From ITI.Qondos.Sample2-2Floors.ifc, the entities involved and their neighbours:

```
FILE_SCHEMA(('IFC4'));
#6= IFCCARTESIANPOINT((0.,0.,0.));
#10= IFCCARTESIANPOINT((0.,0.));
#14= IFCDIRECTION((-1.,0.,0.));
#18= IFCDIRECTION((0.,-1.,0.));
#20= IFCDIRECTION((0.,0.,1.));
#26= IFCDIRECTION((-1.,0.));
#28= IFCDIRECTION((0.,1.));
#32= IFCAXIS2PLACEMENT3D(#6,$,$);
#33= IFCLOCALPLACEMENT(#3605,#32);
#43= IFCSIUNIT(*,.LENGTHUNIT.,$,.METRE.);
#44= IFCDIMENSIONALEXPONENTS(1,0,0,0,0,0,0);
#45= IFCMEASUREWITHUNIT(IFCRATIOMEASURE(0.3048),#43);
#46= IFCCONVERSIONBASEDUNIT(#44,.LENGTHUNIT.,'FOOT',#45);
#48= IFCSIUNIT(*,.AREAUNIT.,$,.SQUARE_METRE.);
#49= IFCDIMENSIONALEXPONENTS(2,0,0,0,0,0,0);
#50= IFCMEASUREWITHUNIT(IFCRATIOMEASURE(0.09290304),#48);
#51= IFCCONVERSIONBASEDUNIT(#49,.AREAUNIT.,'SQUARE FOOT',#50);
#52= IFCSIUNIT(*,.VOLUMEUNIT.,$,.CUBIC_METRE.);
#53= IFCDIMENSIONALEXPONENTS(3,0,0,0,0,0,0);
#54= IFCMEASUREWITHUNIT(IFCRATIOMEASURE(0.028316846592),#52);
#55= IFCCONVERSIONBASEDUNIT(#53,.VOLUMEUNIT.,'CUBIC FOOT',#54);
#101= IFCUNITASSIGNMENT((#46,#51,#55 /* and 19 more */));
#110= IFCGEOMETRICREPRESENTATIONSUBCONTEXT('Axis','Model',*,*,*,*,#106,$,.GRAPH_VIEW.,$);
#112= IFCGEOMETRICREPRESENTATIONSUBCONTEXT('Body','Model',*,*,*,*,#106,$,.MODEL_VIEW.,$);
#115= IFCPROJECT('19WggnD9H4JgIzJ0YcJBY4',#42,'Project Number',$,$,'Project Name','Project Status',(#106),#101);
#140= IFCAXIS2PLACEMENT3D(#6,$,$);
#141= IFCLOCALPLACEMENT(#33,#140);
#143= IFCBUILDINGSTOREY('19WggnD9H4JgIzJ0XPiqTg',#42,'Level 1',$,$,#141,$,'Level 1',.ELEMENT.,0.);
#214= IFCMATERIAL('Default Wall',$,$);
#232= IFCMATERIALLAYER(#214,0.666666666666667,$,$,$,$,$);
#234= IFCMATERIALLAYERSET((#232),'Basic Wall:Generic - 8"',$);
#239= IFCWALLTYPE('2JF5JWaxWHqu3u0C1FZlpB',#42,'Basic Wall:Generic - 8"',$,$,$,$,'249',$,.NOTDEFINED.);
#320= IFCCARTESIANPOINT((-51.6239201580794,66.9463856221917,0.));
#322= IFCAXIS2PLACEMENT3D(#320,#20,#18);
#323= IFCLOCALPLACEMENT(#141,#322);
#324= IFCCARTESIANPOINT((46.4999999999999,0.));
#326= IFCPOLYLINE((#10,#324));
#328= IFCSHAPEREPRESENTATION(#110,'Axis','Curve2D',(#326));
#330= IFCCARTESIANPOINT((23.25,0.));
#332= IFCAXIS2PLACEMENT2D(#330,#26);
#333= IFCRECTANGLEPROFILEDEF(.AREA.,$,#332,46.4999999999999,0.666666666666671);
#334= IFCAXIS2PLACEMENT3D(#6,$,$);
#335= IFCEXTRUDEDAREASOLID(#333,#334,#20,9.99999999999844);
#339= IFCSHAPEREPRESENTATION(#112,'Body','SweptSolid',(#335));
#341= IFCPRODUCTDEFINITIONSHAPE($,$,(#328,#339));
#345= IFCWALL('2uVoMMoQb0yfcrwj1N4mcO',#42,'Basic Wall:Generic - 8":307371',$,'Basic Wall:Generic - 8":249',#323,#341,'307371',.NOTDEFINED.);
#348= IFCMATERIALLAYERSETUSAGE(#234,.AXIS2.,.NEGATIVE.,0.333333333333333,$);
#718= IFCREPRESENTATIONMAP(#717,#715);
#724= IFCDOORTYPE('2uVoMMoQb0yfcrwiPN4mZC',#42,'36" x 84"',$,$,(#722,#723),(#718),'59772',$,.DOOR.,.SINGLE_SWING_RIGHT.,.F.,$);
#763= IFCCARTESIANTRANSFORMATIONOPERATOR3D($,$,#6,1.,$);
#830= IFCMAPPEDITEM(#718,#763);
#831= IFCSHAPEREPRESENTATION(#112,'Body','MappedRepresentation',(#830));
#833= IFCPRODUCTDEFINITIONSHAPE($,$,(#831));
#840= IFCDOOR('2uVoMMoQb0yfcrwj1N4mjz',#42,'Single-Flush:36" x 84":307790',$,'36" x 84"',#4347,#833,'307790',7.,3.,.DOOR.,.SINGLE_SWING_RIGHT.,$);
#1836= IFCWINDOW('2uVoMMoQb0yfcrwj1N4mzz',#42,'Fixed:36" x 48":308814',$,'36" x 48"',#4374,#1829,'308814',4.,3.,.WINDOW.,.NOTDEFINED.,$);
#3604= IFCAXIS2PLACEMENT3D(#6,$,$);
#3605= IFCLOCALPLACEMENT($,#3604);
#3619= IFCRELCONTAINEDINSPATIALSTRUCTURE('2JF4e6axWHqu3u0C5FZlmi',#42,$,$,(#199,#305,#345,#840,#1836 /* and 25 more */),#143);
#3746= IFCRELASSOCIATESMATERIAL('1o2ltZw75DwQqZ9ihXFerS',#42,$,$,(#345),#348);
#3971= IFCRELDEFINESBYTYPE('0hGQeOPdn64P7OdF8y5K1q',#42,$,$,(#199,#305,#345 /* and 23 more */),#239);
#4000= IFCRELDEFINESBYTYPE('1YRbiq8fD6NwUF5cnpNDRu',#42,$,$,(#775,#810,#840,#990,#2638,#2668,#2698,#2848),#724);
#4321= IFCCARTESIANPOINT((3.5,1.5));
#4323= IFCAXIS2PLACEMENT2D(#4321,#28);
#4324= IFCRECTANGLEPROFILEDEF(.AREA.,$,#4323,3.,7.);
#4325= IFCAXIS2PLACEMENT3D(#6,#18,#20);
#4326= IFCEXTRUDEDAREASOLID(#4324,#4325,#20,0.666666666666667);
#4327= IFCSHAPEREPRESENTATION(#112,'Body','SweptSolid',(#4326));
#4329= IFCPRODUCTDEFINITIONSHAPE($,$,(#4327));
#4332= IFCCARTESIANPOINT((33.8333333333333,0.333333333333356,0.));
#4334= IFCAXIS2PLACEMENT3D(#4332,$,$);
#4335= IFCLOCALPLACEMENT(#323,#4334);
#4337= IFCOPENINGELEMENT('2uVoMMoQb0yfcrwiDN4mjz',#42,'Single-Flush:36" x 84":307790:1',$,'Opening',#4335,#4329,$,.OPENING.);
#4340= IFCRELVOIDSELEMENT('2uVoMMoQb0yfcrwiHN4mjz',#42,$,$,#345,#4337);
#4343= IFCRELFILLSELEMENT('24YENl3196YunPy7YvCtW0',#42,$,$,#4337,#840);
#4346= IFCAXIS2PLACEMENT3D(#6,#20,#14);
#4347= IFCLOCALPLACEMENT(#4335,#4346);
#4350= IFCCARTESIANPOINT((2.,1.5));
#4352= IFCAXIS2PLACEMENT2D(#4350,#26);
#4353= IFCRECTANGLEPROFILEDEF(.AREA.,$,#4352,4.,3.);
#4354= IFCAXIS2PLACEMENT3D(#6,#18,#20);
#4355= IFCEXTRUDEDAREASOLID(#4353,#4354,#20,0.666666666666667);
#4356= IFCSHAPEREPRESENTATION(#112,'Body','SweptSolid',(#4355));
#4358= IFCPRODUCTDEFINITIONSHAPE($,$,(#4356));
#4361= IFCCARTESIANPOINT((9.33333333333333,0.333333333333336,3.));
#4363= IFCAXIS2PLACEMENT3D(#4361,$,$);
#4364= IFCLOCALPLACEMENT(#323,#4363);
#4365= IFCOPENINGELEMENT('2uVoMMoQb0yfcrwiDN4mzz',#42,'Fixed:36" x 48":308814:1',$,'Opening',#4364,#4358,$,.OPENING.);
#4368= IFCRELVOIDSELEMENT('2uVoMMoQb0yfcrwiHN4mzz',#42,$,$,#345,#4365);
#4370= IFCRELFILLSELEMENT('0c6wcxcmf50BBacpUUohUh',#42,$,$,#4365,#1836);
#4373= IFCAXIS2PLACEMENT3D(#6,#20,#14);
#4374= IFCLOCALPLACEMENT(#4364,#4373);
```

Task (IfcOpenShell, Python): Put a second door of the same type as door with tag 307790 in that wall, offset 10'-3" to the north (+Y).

```python
import ifcopenshell
import ifcopenshell.api.feature
import ifcopenshell.api.geometry
import ifcopenshell.api.root
import ifcopenshell.geom
import ifcopenshell.util.element
import ifcopenshell.util.placement
import ifcopenshell.util.shape
import ifcopenshell.util.unit

model = ifcopenshell.open("ITI.Qondos.Sample2-2Floors.ifc")
unit_scale = ifcopenshell.util.unit.calculate_unit_scale(model)
settings = ifcopenshell.geom.settings()


def volume(element):
    """Net volume in cubic metres, openings subtracted."""
    shape = ifcopenshell.geom.create_shape(settings, element)
    return ifcopenshell.util.shape.get_volume(shape.geometry)


def reuse_history(source, copy):
    """copy_class also copies each property set's owner history, people and application; keep the originals."""
    for rel in copy.IsDefinedBy:
        if rel.is_a("IfcRelDefinesByProperties") and (history := rel.RelatingPropertyDefinition.OwnerHistory):
            rel.RelatingPropertyDefinition.OwnerHistory = source.OwnerHistory
            ifcopenshell.util.element.remove_deep2(model, history)


door = model.by_guid("2uVoMMoQb0yfcrwj1N4mjz")
opening = door.FillsVoids[0].RelatingOpeningElement
wall = opening.VoidsElements[0].RelatingBuildingElement
before = volume(wall)
shift = ifcopenshell.util.placement.get_local_placement(wall.ObjectPlacement)[:3, 0] * -123 * 0.0254 / unit_scale

# copy_class copies the void relationship, type, container and properties, but no geometry.
new_opening = ifcopenshell.api.root.copy_class(model, product=opening)
new_opening.Representation = ifcopenshell.util.element.copy_deep(
    model, opening.Representation, exclude=["IfcGeometricRepresentationContext", "IfcRepresentationMap"]
)
new_opening.Name = 'Single-Flush:36" x 84"'
new_door = ifcopenshell.api.root.copy_class(model, product=door)
new_door.Representation = ifcopenshell.util.element.copy_deep(
    model, door.Representation, exclude=["IfcGeometricRepresentationContext", "IfcRepresentationMap"]
)
new_door.Name = 'Single-Flush:36" x 84"'
new_door.Tag = None
reuse_history(door, new_door)
ifcopenshell.api.feature.add_filling(model, opening=new_opening, element=new_door)

for old, new in ((opening, new_opening), (door, new_door)):
    matrix = ifcopenshell.util.placement.get_local_placement(old.ObjectPlacement)
    matrix[:3, 3] += shift
    ifcopenshell.api.geometry.edit_object_placement(model, product=new, matrix=matrix, is_si=False)

after = volume(wall)

print(f"wall volume {before:.3f} -> {after:.3f} m3")

model.write("ITI.Qondos.Sample2-2Floors_v2.ifc")
```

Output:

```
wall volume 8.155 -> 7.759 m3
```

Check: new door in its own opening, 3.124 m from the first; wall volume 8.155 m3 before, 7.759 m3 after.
